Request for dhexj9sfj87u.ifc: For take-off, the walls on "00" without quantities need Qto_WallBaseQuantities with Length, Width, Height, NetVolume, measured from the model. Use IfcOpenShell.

First a look at what the model holds.

```python
import ifcopenshell
import ifcopenshell.util.element
import ifcopenshell.util.unit

model = ifcopenshell.open("dhexj9sfj87u.ifc")
print(model.schema)
for unit_type in ("LENGTHUNIT", "AREAUNIT", "VOLUMEUNIT"):
    print(unit_type, ifcopenshell.util.unit.calculate_unit_scale(model, unit_type))
storey = next(s for s in model.by_type("IfcBuildingStorey") if s.Name == "00")
walls = [e for e in ifcopenshell.util.element.get_decomposition(storey) if e.is_a("IfcWall")]
for e in sorted(walls, key=lambda e: e.id()):
    print(e.id(), e.is_a(), e.Name, list(ifcopenshell.util.element.get_psets(e, qtos_only=True)), sep=" | ")
```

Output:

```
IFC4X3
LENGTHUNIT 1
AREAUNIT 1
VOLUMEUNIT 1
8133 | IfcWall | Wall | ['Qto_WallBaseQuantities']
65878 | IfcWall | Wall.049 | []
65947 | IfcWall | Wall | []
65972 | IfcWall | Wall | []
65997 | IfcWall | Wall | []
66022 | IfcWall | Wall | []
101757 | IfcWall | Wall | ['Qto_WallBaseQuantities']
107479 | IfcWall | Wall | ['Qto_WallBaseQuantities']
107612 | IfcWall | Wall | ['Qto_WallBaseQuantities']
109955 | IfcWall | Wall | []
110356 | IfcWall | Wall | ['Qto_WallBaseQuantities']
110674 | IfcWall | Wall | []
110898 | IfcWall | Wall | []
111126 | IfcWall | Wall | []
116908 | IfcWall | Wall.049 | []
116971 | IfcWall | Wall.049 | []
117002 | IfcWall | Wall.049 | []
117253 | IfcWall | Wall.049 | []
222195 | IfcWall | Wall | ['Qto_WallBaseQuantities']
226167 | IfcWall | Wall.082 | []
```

```python
import ifcopenshell
import ifcopenshell.api.pset
import ifcopenshell.geom
import ifcopenshell.util.element
import ifcopenshell.util.shape
import ifcopenshell.util.unit

model = ifcopenshell.open("dhexj9sfj87u.ifc")
unit_scale = ifcopenshell.util.unit.calculate_unit_scale(model)
volume_scale = ifcopenshell.util.unit.calculate_unit_scale(model, "VOLUMEUNIT")
settings = ifcopenshell.geom.settings()

storey = next(s for s in model.by_type("IfcBuildingStorey") if s.Name == "00")
walls = [e for e in ifcopenshell.util.element.get_decomposition(storey) if e.is_a("IfcWall")]

for e in sorted(walls, key=lambda e: e.id()):
    if ifcopenshell.util.element.get_psets(e, qtos_only=True, should_inherit=False):
        continue
    # Geometry comes back in metres, in the element's own axes.
    shape = ifcopenshell.geom.create_shape(settings, e)
    values = {
        "Length": ifcopenshell.util.shape.get_x(shape.geometry) / unit_scale,
        "Width": ifcopenshell.util.shape.get_y(shape.geometry) / unit_scale,
        "Height": ifcopenshell.util.shape.get_z(shape.geometry) / unit_scale,
        "NetVolume": ifcopenshell.util.shape.get_volume(shape.geometry) / volume_scale,
    }
    qto = ifcopenshell.api.pset.add_qto(model, product=e, name="Qto_WallBaseQuantities")
    ifcopenshell.api.pset.edit_qto(model, qto=qto, properties=values)
    print(e.id(), {k: round(v, 3) for k, v in values.items()})

model.write("dhexj9sfj87u_updated.ifc")
```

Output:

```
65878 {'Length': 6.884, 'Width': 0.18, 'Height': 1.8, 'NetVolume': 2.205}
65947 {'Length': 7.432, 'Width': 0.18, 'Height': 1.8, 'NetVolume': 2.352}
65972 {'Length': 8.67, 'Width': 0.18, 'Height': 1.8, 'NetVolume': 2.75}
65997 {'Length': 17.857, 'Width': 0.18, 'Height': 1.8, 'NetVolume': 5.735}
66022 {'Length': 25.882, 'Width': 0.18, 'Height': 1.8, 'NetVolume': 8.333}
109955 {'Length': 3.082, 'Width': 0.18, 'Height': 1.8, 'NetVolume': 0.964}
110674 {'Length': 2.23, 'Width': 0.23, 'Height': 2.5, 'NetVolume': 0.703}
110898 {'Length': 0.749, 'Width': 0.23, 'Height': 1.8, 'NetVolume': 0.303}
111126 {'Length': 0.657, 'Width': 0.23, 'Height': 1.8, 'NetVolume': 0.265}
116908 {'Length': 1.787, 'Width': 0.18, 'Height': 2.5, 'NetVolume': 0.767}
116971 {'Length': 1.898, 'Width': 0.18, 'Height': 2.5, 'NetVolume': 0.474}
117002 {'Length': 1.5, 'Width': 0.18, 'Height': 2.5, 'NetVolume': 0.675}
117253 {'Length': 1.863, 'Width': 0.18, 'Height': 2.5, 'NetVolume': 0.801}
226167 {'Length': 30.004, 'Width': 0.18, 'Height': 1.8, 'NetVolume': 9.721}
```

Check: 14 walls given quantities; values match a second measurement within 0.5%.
